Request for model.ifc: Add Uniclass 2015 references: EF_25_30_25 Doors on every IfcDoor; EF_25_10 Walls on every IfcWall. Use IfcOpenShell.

First a look at what the model holds.

```python
import ifcopenshell

model = ifcopenshell.open("model.ifc")
print(model.schema)
print("classifications:", [c.Name for c in model.by_type("IfcClassification")])
for ifc_class in ("IfcDoor", "IfcRoof", "IfcStair", "IfcWall", "IfcWindow"):
    print(ifc_class, len(model.by_type(ifc_class)))
```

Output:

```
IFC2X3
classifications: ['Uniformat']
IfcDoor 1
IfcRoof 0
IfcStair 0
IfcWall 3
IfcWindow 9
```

```python
import ifcopenshell
import ifcopenshell.api.classification

model = ifcopenshell.open("model.ifc")

# IFC2X3 requires Source and Edition and has no link from the project to the system.
system = model.create_entity("IfcClassification", Source="NBS", Edition="2015", Name="Uniclass 2015")

codes = {
    "IfcDoor": ("EF_25_30_25", "Doors"),
    "IfcWall": ("EF_25_10", "Walls"),
}
for ifc_class, (code, name) in codes.items():
    products = model.by_type(ifc_class)
    ifcopenshell.api.classification.add_reference(
        model, products=products, classification=system, identification=code, name=name
    )
    print(code, len(products))

model.write("model_updated.ifc")
```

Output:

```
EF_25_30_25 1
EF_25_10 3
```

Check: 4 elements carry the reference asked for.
